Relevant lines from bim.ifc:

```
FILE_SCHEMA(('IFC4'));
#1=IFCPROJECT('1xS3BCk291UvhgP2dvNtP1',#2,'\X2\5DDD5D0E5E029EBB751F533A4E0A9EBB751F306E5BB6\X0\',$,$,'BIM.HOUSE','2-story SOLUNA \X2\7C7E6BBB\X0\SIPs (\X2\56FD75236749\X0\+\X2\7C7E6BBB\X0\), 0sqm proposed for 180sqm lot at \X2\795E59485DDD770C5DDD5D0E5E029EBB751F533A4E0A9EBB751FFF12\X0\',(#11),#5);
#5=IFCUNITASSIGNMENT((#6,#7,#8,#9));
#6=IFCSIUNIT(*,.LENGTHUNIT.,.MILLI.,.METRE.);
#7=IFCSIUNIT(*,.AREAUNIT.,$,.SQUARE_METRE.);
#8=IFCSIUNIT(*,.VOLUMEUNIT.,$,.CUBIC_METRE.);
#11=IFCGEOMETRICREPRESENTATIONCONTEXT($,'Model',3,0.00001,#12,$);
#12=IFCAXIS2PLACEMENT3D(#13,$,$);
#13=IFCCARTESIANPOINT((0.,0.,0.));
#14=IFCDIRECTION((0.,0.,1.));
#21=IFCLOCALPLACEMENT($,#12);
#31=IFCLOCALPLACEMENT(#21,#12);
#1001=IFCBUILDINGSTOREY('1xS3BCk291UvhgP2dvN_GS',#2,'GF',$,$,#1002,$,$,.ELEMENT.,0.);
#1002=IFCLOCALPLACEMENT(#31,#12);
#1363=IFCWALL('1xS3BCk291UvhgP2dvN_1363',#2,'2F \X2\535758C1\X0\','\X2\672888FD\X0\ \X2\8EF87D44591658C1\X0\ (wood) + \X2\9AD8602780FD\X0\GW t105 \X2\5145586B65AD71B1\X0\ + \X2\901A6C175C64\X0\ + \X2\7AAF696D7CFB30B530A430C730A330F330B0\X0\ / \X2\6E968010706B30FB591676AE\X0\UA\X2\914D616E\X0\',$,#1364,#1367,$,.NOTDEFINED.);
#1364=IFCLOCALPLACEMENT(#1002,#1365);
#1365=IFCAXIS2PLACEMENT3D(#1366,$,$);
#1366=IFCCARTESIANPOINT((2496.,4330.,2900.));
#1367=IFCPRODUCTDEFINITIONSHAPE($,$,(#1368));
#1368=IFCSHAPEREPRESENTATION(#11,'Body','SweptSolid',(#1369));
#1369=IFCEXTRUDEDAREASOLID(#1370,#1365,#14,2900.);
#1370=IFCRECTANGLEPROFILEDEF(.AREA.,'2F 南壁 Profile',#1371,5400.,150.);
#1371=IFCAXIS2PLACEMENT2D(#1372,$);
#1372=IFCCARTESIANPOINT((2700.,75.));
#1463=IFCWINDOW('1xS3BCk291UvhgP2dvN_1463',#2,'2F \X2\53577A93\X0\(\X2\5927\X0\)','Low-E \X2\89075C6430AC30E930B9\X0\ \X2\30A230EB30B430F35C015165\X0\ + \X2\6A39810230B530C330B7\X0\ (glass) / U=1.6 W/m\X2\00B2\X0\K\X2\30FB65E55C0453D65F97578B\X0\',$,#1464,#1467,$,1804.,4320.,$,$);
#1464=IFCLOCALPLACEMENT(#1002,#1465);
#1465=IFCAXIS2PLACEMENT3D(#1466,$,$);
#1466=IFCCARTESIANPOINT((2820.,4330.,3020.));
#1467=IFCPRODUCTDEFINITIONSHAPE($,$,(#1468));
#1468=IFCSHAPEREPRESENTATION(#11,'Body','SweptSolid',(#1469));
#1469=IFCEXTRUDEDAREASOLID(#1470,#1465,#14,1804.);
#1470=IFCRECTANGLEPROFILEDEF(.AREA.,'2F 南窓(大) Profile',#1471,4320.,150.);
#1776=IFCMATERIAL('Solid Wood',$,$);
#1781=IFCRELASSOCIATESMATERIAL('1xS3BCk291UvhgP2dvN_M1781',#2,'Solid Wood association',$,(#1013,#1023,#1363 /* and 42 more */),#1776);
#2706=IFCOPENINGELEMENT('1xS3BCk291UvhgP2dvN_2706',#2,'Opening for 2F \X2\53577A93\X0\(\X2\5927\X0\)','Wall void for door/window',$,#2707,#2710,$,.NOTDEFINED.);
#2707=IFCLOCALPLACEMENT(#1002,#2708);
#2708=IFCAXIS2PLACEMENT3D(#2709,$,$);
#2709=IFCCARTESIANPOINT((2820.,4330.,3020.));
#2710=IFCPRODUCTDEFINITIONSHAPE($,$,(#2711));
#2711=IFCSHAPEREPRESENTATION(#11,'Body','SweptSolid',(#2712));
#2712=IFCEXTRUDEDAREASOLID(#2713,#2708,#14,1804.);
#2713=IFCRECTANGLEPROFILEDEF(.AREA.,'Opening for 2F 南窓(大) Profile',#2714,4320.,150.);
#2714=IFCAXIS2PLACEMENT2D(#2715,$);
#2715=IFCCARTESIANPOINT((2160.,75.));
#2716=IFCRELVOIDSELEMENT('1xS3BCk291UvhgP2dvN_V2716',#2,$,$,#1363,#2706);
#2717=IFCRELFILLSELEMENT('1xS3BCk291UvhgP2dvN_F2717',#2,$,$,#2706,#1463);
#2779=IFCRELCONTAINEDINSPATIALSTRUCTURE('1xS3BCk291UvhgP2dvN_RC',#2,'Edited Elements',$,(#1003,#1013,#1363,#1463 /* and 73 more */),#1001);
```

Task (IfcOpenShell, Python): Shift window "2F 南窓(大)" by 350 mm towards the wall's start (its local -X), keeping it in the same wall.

```python
import ifcopenshell
import ifcopenshell.api.geometry
import ifcopenshell.util.placement

model = ifcopenshell.open("bim.ifc")

window = model.by_guid("1xS3BCk291UvhgP2dvN_1463")
opening = window.FillsVoids[0].RelatingOpeningElement
wall = opening.VoidsElements[0].RelatingBuildingElement

wall_matrix = ifcopenshell.util.placement.get_local_placement(wall.ObjectPlacement)
shift = wall_matrix[:3, 0] * -350.0
before = ifcopenshell.util.placement.get_local_placement(window.ObjectPlacement)[:3, 3].copy()

# The window is not placed relative to its opening, so move both.
for product in (opening, window):
    matrix = ifcopenshell.util.placement.get_local_placement(product.ObjectPlacement)
    matrix[:3, 3] += shift
    ifcopenshell.api.geometry.edit_object_placement(model, product=product, matrix=matrix, is_si=False)

after = ifcopenshell.util.placement.get_local_placement(window.ObjectPlacement)[:3, 3]
print("window moved by", (after - before).round(3) + 0.0)

model.write("bim_v2.ifc")
```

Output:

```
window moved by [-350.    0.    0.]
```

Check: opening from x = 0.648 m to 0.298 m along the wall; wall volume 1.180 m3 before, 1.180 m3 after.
